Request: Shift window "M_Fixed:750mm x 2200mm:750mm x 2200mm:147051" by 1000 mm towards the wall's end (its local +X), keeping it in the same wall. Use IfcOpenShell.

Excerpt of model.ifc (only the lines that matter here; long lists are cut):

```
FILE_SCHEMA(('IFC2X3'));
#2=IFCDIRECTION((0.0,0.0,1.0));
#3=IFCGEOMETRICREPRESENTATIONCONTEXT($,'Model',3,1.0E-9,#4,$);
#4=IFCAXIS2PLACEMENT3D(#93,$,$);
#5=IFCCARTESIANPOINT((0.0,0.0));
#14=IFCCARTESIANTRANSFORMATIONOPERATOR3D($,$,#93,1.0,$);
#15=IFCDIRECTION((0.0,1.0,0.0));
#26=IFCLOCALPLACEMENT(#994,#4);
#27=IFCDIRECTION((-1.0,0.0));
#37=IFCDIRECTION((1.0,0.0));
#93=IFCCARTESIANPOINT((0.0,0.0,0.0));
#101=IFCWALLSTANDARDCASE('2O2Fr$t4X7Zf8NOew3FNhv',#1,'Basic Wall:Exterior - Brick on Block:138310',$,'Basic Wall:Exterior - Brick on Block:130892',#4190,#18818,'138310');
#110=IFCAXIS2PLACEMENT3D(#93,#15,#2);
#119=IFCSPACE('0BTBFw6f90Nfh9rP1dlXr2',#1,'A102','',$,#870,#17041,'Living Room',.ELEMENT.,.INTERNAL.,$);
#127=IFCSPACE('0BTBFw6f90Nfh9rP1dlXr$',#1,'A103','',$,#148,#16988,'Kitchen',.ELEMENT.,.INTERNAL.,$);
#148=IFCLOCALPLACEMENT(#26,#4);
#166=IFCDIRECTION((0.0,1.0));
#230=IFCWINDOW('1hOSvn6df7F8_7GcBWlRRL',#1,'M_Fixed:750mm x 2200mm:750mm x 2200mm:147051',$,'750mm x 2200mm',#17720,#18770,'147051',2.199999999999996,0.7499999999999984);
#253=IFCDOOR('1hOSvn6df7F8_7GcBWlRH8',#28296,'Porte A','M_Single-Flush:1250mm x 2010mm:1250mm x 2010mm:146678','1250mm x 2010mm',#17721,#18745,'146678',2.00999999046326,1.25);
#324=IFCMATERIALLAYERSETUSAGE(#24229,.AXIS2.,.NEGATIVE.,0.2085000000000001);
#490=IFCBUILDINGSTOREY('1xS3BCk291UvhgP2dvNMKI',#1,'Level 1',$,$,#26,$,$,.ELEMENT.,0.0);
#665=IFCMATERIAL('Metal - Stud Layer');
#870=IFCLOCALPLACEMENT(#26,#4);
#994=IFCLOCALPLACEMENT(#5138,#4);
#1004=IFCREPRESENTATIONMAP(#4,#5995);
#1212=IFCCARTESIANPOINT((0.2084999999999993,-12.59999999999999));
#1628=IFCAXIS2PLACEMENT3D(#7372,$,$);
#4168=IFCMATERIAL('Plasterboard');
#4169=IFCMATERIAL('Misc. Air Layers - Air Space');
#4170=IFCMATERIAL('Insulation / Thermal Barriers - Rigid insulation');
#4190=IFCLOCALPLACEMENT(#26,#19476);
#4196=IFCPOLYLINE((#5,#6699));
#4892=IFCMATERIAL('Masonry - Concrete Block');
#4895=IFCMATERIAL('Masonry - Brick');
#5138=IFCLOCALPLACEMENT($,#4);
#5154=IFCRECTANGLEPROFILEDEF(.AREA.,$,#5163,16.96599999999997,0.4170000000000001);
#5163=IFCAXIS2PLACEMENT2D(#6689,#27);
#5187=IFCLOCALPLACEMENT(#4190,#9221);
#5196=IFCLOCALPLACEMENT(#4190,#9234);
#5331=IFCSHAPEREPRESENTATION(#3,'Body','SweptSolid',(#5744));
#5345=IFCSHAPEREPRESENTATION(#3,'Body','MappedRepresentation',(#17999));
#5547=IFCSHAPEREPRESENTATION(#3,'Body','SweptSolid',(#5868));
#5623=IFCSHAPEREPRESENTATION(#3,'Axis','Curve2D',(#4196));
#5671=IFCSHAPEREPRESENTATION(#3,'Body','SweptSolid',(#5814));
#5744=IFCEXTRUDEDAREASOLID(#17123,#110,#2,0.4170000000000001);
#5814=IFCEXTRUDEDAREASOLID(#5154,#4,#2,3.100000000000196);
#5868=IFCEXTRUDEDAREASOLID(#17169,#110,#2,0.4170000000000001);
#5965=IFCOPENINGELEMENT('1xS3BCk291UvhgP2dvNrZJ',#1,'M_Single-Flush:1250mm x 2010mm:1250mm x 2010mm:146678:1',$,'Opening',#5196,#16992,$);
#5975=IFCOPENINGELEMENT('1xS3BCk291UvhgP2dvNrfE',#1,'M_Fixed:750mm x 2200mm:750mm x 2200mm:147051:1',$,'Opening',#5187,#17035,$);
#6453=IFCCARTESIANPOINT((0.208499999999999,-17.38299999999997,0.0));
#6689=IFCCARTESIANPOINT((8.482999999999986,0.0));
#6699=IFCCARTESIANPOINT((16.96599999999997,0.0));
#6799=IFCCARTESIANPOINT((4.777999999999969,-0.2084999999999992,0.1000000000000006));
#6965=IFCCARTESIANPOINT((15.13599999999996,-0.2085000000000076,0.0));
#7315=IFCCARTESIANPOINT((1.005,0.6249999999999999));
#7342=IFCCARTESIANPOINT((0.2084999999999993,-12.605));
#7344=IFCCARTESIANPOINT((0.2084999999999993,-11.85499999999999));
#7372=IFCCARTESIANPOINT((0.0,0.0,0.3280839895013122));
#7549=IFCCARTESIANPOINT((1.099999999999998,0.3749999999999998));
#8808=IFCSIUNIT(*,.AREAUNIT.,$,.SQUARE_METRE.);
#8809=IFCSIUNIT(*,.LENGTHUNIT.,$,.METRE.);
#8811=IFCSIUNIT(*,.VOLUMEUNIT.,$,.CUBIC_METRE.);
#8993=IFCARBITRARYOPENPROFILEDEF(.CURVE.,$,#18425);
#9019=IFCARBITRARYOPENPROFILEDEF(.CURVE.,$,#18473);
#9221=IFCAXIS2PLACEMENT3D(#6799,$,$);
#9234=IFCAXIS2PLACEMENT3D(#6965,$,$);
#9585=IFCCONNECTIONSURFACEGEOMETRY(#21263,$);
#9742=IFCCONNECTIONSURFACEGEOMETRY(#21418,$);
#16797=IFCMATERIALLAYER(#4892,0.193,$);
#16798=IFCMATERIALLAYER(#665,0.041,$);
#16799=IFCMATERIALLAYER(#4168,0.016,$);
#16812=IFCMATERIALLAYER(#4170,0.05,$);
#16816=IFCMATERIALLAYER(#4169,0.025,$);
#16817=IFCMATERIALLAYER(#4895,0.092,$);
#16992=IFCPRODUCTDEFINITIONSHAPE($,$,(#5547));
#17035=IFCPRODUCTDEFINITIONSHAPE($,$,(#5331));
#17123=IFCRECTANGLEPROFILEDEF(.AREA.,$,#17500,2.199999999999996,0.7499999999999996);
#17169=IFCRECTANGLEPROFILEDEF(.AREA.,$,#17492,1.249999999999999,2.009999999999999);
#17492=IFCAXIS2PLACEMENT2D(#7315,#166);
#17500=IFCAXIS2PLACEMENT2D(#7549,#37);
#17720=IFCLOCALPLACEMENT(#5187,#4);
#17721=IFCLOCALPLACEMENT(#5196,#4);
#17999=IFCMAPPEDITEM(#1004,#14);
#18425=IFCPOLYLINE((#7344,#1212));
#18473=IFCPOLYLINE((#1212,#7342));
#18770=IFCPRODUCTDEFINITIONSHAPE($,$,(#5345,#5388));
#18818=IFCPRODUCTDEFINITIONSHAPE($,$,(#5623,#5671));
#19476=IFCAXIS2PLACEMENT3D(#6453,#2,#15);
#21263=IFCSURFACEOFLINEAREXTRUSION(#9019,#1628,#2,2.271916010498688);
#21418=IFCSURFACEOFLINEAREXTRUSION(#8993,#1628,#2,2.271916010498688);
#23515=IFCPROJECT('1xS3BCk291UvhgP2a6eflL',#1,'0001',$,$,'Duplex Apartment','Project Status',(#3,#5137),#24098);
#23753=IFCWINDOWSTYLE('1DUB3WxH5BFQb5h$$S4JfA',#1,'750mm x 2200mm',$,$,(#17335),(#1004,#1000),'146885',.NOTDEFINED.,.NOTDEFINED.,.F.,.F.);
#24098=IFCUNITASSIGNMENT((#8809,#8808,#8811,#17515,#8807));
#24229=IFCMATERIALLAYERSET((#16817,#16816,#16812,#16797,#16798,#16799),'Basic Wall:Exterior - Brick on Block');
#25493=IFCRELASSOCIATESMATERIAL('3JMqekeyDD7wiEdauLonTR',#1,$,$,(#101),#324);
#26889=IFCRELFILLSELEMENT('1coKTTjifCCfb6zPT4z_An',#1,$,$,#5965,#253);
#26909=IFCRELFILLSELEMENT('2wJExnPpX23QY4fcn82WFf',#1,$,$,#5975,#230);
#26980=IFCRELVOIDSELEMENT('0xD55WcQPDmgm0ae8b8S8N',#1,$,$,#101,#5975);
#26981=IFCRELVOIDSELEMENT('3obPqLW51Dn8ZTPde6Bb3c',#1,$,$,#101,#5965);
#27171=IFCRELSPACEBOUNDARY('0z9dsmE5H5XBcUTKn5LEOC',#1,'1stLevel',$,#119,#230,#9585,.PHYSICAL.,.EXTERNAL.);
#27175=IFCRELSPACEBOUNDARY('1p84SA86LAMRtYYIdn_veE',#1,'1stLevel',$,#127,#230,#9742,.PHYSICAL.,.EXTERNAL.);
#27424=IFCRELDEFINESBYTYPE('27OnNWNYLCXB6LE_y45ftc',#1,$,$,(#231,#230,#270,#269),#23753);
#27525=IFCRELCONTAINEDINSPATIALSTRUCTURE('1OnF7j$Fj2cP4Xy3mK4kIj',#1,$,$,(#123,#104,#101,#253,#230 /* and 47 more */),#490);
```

```python
import numpy as np
import ifcopenshell
import ifcopenshell.api.geometry
import ifcopenshell.util.placement
import ifcopenshell.util.unit

model = ifcopenshell.open("model.ifc")
unit_scale = ifcopenshell.util.unit.calculate_unit_scale(model)

window = model.by_guid("1hOSvn6df7F8_7GcBWlRRL")
opening = window.FillsVoids[0].RelatingOpeningElement
wall = opening.VoidsElements[0].RelatingBuildingElement

wall_matrix = ifcopenshell.util.placement.get_local_placement(wall.ObjectPlacement)
shift = wall_matrix[:3, 0] * 1 / unit_scale
before = ifcopenshell.util.placement.get_local_placement(window.ObjectPlacement)[:3, 3].copy()

# The window is placed relative to its opening, so it follows when the opening moves.
matrix = ifcopenshell.util.placement.get_local_placement(opening.ObjectPlacement)
matrix[:3, 3] += shift
ifcopenshell.api.geometry.edit_object_placement(
    model, product=opening, matrix=matrix, is_si=False, should_transform_children=True
)

# Space boundary surfaces are stored in each space's coordinates; move them too.
for rel in window.ProvidesBoundaries:
    if not rel.ConnectionGeometry:
        continue
    surface = rel.ConnectionGeometry.SurfaceOnRelatingElement
    space_matrix = ifcopenshell.util.placement.get_local_placement(rel.RelatingSpace.ObjectPlacement)
    point = np.array(surface.Position.Location.Coordinates) + space_matrix[:3, :3].T @ shift
    surface.Position = model.createIfcAxis2Placement3D(
        model.createIfcCartesianPoint(point.tolist()), surface.Position.Axis, surface.Position.RefDirection
    )

after = ifcopenshell.util.placement.get_local_placement(window.ObjectPlacement)[:3, 3]
print("window moved by", (after - before).round(3) + 0.0)

model.write("model_updated.ifc")
```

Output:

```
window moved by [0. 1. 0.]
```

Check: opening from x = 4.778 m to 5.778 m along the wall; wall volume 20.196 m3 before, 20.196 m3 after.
